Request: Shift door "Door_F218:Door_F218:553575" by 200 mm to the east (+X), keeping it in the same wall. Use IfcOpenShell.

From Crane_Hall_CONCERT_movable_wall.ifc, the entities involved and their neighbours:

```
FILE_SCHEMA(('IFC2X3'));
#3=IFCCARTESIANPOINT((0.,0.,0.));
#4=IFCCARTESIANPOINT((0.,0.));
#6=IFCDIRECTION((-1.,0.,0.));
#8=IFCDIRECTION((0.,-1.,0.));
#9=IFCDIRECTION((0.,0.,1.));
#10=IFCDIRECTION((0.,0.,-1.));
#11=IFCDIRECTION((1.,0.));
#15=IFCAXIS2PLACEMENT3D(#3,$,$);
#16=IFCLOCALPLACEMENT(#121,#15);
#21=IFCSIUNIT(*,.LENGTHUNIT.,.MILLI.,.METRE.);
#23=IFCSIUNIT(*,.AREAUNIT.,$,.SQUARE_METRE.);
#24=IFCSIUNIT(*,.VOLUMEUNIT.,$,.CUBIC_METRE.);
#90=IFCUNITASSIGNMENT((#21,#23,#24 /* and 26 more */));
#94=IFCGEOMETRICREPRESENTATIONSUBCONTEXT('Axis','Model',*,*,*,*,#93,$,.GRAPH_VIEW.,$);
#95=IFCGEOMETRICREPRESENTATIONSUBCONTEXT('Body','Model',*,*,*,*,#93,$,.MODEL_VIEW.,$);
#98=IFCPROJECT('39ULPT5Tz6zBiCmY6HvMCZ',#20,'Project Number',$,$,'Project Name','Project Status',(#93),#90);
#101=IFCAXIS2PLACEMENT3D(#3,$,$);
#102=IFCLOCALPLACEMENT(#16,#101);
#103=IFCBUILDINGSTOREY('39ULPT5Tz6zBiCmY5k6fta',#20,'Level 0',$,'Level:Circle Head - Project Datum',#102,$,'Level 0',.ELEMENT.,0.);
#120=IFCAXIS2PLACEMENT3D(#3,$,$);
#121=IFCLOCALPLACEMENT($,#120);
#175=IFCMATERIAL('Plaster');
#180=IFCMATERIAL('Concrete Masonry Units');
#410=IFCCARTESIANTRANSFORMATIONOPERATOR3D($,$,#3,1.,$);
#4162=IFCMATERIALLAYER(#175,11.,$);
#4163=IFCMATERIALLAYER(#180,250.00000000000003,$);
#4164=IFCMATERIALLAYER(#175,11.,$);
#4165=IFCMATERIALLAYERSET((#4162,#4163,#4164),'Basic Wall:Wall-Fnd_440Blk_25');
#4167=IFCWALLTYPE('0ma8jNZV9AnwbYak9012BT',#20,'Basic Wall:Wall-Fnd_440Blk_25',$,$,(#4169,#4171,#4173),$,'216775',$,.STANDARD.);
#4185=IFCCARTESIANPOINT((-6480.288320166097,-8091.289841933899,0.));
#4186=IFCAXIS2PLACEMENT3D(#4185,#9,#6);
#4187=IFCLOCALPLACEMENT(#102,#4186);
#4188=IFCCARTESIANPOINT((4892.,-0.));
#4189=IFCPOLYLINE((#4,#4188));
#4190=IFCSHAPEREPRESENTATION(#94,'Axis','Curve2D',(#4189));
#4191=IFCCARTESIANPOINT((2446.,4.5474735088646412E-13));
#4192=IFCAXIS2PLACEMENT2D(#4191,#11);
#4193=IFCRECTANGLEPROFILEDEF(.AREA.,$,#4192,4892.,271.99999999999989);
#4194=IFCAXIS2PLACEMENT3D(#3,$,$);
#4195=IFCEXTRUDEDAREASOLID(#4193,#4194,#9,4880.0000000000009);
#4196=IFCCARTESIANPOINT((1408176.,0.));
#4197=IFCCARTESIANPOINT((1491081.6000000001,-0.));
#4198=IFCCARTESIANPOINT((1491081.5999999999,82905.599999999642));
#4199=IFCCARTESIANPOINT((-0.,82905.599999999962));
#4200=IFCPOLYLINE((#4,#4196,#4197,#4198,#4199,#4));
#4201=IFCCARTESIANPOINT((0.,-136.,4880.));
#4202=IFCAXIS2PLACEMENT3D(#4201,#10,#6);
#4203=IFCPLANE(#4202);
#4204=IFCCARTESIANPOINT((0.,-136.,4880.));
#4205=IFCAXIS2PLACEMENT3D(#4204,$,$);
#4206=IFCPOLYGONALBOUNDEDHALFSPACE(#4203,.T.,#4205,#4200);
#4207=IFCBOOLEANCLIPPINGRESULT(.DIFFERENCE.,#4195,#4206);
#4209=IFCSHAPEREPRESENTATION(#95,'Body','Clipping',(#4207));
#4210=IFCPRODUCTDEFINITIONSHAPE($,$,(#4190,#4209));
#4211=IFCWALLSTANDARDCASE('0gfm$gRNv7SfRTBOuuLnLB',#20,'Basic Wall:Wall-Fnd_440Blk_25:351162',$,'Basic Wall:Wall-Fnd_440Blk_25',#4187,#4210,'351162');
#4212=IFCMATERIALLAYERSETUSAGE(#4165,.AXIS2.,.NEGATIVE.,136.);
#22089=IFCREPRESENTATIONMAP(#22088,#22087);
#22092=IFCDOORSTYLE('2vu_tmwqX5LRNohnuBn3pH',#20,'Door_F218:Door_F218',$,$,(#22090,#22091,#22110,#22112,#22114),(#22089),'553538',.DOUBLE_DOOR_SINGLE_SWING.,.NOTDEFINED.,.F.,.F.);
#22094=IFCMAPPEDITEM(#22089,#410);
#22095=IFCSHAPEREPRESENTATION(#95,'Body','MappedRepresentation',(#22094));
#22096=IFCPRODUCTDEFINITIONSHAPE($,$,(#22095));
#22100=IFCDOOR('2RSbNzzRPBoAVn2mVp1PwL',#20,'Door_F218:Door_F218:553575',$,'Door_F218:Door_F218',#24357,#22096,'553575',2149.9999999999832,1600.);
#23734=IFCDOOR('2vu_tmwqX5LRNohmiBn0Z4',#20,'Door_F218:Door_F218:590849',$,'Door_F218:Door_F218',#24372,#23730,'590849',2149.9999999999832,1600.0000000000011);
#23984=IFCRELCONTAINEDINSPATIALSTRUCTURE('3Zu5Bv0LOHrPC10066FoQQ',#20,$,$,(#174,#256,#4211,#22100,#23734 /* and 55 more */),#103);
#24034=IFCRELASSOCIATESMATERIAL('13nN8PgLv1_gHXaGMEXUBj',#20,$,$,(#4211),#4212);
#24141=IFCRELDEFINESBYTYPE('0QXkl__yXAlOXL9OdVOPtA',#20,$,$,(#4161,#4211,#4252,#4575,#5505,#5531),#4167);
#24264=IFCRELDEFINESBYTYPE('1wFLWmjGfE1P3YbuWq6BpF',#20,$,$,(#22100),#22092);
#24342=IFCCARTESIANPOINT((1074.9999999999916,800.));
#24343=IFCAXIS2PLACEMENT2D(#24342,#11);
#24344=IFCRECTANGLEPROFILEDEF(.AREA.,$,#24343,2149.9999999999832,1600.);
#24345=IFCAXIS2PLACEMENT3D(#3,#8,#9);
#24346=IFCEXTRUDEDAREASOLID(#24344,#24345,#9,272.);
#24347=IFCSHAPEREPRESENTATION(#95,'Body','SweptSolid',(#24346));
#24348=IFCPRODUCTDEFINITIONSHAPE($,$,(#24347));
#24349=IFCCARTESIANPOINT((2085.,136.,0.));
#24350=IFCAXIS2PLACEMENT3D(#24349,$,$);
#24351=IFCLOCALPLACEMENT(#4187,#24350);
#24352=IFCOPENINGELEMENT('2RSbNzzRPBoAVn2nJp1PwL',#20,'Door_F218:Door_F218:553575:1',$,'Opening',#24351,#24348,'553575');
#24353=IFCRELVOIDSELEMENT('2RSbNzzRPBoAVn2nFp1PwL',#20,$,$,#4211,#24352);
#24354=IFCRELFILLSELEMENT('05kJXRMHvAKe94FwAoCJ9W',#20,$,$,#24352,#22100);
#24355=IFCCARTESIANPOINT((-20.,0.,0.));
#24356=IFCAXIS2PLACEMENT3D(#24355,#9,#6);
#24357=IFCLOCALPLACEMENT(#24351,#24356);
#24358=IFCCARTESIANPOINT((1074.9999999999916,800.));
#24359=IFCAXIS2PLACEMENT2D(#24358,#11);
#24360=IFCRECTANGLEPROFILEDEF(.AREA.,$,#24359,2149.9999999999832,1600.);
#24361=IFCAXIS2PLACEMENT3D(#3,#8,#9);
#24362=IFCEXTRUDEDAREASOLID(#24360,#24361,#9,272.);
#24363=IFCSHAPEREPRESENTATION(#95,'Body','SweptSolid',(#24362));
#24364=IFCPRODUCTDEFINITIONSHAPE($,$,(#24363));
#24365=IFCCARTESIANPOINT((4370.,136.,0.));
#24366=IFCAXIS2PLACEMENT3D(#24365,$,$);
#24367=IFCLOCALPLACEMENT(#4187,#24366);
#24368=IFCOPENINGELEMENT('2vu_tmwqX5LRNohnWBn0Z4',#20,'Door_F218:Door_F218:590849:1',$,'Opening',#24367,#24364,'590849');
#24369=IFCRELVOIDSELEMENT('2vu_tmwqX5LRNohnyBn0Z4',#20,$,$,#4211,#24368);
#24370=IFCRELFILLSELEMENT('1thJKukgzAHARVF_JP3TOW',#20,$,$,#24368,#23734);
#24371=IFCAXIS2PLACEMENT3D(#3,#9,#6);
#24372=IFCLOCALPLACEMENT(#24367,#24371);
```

```python
import ifcopenshell
import ifcopenshell.api.geometry
import ifcopenshell.util.placement
import ifcopenshell.util.unit

model = ifcopenshell.open("Crane_Hall_CONCERT_movable_wall.ifc")
unit_scale = ifcopenshell.util.unit.calculate_unit_scale(model)

door = model.by_guid("2RSbNzzRPBoAVn2mVp1PwL")
opening = door.FillsVoids[0].RelatingOpeningElement
wall = opening.VoidsElements[0].RelatingBuildingElement

wall_matrix = ifcopenshell.util.placement.get_local_placement(wall.ObjectPlacement)
shift = wall_matrix[:3, 0] * -0.2 / unit_scale
before = ifcopenshell.util.placement.get_local_placement(door.ObjectPlacement)[:3, 3].copy()

# The door is placed relative to its opening, so it follows when the opening moves.
matrix = ifcopenshell.util.placement.get_local_placement(opening.ObjectPlacement)
matrix[:3, 3] += shift
ifcopenshell.api.geometry.edit_object_placement(
    model, product=opening, matrix=matrix, is_si=False, should_transform_children=True
)

after = ifcopenshell.util.placement.get_local_placement(door.ObjectPlacement)[:3, 3]
print("door moved by", (after - before).round(3) + 0.0)

model.write("Crane_Hall_CONCERT_movable_wall_edited.ifc")
```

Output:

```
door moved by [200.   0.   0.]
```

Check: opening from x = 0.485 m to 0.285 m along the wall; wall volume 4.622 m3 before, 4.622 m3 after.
